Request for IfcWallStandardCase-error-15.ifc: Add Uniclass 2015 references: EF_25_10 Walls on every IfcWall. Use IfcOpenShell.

First a look at what the model holds.

```python
import ifcopenshell

model = ifcopenshell.open("IfcWallStandardCase-error-15.ifc")
print(model.schema)
print("classifications:", [c.Name for c in model.by_type("IfcClassification")])
for ifc_class in ("IfcDoor", "IfcRoof", "IfcStair", "IfcWall", "IfcWindow"):
    print(ifc_class, len(model.by_type(ifc_class)))
```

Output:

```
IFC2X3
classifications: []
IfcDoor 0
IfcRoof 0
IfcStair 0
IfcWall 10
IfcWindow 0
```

```python
import ifcopenshell
import ifcopenshell.api.classification

model = ifcopenshell.open("IfcWallStandardCase-error-15.ifc")

# IFC2X3 requires Source and Edition and has no link from the project to the system.
system = model.create_entity("IfcClassification", Source="NBS", Edition="2015", Name="Uniclass 2015")

codes = {
    "IfcWall": ("EF_25_10", "Walls"),
}
for ifc_class, (code, name) in codes.items():
    products = model.by_type(ifc_class)
    ifcopenshell.api.classification.add_reference(
        model, products=products, classification=system, identification=code, name=name
    )
    print(code, len(products))

model.write("IfcWallStandardCase-error-15_v2.ifc")
```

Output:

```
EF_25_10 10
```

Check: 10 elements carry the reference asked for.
